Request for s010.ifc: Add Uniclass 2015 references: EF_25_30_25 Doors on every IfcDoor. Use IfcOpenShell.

First a look at what the model holds.

```python
import ifcopenshell

model = ifcopenshell.open("s010.ifc")
print(model.schema)
print("classifications:", [c.Name for c in model.by_type("IfcClassification")])
for ifc_class in ("IfcDoor", "IfcRoof", "IfcStair", "IfcWall", "IfcWindow"):
    print(ifc_class, len(model.by_type(ifc_class)))
```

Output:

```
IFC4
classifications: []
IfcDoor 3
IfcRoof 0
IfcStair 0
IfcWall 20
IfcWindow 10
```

```python
import ifcopenshell
import ifcopenshell.api.classification

model = ifcopenshell.open("s010.ifc")

system = ifcopenshell.api.classification.add_classification(model, classification="Uniclass 2015")

codes = {
    "IfcDoor": ("EF_25_30_25", "Doors"),
}
for ifc_class, (code, name) in codes.items():
    products = model.by_type(ifc_class)
    ifcopenshell.api.classification.add_reference(
        model, products=products, classification=system, identification=code, name=name
    )
    print(code, len(products))

model.write("s010_edited.ifc")
```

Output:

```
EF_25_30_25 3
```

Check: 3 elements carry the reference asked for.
